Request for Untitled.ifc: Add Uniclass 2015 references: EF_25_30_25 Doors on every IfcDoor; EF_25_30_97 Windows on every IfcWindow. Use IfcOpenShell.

First a look at what the model holds.

```python
import ifcopenshell

model = ifcopenshell.open("Untitled.ifc")
print(model.schema)
print("classifications:", [c.Name for c in model.by_type("IfcClassification")])
for ifc_class in ("IfcDoor", "IfcRoof", "IfcStair", "IfcWall", "IfcWindow"):
    print(ifc_class, len(model.by_type(ifc_class)))
```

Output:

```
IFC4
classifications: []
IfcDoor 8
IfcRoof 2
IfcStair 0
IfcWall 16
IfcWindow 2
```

```python
import ifcopenshell
import ifcopenshell.api.classification

model = ifcopenshell.open("Untitled.ifc")

system = ifcopenshell.api.classification.add_classification(model, classification="Uniclass 2015")

codes = {
    "IfcDoor": ("EF_25_30_25", "Doors"),
    "IfcWindow": ("EF_25_30_97", "Windows"),
}
for ifc_class, (code, name) in codes.items():
    products = model.by_type(ifc_class)
    ifcopenshell.api.classification.add_reference(
        model, products=products, classification=system, identification=code, name=name
    )
    print(code, len(products))

model.write("Untitled_edited.ifc")
```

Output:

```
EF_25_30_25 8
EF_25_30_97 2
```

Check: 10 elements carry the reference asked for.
